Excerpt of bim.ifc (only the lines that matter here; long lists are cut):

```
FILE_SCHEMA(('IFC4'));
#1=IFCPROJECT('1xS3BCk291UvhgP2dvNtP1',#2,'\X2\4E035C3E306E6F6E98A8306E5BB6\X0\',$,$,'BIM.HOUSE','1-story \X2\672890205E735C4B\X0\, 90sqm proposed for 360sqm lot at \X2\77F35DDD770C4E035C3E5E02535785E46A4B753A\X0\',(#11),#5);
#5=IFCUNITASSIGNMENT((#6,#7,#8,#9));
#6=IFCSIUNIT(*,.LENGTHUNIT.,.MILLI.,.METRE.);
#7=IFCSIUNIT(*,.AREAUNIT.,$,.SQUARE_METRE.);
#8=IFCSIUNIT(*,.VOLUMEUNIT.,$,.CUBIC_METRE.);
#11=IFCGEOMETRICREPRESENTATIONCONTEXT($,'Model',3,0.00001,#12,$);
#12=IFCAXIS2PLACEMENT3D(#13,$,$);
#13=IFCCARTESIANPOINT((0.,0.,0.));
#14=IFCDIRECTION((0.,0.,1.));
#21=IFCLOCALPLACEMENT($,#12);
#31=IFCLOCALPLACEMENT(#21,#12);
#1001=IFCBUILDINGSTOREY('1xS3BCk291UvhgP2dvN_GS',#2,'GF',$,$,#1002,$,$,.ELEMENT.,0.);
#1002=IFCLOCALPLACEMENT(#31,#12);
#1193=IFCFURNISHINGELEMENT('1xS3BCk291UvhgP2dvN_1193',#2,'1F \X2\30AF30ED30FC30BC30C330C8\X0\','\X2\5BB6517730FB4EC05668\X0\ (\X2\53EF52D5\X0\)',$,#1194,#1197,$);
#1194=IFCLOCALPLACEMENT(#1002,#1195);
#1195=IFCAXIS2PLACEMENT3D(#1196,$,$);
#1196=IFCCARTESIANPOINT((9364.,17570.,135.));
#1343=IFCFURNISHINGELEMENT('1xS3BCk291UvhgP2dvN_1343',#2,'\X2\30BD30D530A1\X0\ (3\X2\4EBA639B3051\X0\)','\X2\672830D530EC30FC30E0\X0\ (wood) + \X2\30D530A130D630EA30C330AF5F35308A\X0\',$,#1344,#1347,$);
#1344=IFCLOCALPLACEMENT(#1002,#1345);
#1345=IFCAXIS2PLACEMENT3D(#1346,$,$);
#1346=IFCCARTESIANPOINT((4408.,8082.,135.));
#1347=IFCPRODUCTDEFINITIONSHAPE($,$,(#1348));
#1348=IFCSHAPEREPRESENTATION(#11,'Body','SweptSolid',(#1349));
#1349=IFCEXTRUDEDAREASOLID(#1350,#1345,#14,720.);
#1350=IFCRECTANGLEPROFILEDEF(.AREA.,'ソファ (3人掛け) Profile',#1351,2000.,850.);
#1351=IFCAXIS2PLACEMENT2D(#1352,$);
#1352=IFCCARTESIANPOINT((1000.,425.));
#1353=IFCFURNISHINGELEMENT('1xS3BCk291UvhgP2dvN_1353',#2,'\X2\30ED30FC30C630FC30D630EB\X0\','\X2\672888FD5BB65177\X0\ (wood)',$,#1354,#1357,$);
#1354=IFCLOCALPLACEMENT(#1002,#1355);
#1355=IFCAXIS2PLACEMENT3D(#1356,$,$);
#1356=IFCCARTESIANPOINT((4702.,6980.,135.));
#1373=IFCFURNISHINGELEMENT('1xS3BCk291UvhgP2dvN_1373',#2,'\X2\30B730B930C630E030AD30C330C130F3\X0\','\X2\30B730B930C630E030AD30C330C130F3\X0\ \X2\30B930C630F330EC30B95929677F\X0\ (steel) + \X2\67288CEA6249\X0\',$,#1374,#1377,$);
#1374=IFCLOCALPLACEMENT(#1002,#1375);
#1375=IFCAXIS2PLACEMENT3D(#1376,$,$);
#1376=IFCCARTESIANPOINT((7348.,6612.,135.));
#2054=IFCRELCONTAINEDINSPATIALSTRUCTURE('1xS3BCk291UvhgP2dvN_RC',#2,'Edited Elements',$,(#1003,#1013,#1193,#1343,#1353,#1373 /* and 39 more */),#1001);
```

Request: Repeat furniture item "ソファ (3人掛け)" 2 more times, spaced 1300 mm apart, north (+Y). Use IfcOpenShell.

```python
import numpy as np
import ifcopenshell
import ifcopenshell.api.geometry
import ifcopenshell.api.root
import ifcopenshell.util.element
import ifcopenshell.util.placement
import ifcopenshell.util.unit

model = ifcopenshell.open("bim.ifc")
unit_scale = ifcopenshell.util.unit.calculate_unit_scale(model)


def reuse_history(source, copy):
    """copy_class also copies each property set's owner history, people and application; keep the originals."""
    for rel in copy.IsDefinedBy:
        if rel.is_a("IfcRelDefinesByProperties") and (history := rel.RelatingPropertyDefinition.OwnerHistory):
            rel.RelatingPropertyDefinition.OwnerHistory = source.OwnerHistory
            ifcopenshell.util.element.remove_deep2(model, history)


source = model.by_guid("1xS3BCk291UvhgP2dvN_1343")
base = ifcopenshell.util.placement.get_local_placement(source.ObjectPlacement)
step = np.array([0.0, 1.0, 0.0]) * 1.3 / unit_scale

for i in range(1, 3):
    copy = ifcopenshell.api.root.copy_class(model, product=source)
    copy.Representation = ifcopenshell.util.element.copy_deep(
        model, source.Representation, exclude=["IfcGeometricRepresentationContext", "IfcRepresentationMap"]
    )
    reuse_history(source, copy)
    matrix = base.copy()
    matrix[:3, 3] += i * step
    print("added at", matrix[:3, 3].round(3) + 0.0)
    ifcopenshell.api.geometry.edit_object_placement(model, product=copy, matrix=matrix, is_si=False)

model.write("bim_rev.ifc")
```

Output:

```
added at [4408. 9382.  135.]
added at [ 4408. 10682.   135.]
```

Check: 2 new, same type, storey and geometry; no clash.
